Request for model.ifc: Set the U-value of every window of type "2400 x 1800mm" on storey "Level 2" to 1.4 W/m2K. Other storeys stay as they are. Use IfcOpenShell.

First a look at what the model holds.

```python
import ifcopenshell
import ifcopenshell.util.element

model = ifcopenshell.open("model.ifc")
print(model.schema)
storey = next(s for s in model.by_type("IfcBuildingStorey") if s.Name == "Level 2")
windows = [e for e in ifcopenshell.util.element.get_decomposition(storey) if e.is_a("IfcWindow")]
seen = {}
for e in windows:
    element_type = ifcopenshell.util.element.get_type(e)
    key = (element_type.Name if element_type != e and element_type else None, ifcopenshell.util.element.get_pset(e, "Pset_WindowCommon", "ThermalTransmittance"))
    seen[key] = seen.get(key, 0) + 1
for (name, value), count in sorted(seen.items(), key=str):
    print(count, "x", name, "|", value)
```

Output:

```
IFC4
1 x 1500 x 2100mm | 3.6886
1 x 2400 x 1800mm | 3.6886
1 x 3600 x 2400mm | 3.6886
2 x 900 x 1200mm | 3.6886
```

```python
import ifcopenshell
import ifcopenshell.api.pset
import ifcopenshell.util.element

model = ifcopenshell.open("model.ifc")

storey = next(s for s in model.by_type("IfcBuildingStorey") if s.Name == "Level 2")
windows = [e for e in ifcopenshell.util.element.get_decomposition(storey) if e.is_a("IfcWindow")]

count = 0
for e in windows:
    element_type = ifcopenshell.util.element.get_type(e)
    if element_type in (None, e) or element_type.Name != "2400 x 1800mm":
        continue
    # add_pset returns the element's existing set when there is one.
    pset = ifcopenshell.api.pset.add_pset(model, product=e, name="Pset_WindowCommon")
    ifcopenshell.api.pset.edit_pset(model, pset=pset, properties={"ThermalTransmittance": 1.4})
    count += 1

print(count, "windows updated")

model.write("model_v2.ifc")
```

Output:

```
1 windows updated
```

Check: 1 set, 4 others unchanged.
